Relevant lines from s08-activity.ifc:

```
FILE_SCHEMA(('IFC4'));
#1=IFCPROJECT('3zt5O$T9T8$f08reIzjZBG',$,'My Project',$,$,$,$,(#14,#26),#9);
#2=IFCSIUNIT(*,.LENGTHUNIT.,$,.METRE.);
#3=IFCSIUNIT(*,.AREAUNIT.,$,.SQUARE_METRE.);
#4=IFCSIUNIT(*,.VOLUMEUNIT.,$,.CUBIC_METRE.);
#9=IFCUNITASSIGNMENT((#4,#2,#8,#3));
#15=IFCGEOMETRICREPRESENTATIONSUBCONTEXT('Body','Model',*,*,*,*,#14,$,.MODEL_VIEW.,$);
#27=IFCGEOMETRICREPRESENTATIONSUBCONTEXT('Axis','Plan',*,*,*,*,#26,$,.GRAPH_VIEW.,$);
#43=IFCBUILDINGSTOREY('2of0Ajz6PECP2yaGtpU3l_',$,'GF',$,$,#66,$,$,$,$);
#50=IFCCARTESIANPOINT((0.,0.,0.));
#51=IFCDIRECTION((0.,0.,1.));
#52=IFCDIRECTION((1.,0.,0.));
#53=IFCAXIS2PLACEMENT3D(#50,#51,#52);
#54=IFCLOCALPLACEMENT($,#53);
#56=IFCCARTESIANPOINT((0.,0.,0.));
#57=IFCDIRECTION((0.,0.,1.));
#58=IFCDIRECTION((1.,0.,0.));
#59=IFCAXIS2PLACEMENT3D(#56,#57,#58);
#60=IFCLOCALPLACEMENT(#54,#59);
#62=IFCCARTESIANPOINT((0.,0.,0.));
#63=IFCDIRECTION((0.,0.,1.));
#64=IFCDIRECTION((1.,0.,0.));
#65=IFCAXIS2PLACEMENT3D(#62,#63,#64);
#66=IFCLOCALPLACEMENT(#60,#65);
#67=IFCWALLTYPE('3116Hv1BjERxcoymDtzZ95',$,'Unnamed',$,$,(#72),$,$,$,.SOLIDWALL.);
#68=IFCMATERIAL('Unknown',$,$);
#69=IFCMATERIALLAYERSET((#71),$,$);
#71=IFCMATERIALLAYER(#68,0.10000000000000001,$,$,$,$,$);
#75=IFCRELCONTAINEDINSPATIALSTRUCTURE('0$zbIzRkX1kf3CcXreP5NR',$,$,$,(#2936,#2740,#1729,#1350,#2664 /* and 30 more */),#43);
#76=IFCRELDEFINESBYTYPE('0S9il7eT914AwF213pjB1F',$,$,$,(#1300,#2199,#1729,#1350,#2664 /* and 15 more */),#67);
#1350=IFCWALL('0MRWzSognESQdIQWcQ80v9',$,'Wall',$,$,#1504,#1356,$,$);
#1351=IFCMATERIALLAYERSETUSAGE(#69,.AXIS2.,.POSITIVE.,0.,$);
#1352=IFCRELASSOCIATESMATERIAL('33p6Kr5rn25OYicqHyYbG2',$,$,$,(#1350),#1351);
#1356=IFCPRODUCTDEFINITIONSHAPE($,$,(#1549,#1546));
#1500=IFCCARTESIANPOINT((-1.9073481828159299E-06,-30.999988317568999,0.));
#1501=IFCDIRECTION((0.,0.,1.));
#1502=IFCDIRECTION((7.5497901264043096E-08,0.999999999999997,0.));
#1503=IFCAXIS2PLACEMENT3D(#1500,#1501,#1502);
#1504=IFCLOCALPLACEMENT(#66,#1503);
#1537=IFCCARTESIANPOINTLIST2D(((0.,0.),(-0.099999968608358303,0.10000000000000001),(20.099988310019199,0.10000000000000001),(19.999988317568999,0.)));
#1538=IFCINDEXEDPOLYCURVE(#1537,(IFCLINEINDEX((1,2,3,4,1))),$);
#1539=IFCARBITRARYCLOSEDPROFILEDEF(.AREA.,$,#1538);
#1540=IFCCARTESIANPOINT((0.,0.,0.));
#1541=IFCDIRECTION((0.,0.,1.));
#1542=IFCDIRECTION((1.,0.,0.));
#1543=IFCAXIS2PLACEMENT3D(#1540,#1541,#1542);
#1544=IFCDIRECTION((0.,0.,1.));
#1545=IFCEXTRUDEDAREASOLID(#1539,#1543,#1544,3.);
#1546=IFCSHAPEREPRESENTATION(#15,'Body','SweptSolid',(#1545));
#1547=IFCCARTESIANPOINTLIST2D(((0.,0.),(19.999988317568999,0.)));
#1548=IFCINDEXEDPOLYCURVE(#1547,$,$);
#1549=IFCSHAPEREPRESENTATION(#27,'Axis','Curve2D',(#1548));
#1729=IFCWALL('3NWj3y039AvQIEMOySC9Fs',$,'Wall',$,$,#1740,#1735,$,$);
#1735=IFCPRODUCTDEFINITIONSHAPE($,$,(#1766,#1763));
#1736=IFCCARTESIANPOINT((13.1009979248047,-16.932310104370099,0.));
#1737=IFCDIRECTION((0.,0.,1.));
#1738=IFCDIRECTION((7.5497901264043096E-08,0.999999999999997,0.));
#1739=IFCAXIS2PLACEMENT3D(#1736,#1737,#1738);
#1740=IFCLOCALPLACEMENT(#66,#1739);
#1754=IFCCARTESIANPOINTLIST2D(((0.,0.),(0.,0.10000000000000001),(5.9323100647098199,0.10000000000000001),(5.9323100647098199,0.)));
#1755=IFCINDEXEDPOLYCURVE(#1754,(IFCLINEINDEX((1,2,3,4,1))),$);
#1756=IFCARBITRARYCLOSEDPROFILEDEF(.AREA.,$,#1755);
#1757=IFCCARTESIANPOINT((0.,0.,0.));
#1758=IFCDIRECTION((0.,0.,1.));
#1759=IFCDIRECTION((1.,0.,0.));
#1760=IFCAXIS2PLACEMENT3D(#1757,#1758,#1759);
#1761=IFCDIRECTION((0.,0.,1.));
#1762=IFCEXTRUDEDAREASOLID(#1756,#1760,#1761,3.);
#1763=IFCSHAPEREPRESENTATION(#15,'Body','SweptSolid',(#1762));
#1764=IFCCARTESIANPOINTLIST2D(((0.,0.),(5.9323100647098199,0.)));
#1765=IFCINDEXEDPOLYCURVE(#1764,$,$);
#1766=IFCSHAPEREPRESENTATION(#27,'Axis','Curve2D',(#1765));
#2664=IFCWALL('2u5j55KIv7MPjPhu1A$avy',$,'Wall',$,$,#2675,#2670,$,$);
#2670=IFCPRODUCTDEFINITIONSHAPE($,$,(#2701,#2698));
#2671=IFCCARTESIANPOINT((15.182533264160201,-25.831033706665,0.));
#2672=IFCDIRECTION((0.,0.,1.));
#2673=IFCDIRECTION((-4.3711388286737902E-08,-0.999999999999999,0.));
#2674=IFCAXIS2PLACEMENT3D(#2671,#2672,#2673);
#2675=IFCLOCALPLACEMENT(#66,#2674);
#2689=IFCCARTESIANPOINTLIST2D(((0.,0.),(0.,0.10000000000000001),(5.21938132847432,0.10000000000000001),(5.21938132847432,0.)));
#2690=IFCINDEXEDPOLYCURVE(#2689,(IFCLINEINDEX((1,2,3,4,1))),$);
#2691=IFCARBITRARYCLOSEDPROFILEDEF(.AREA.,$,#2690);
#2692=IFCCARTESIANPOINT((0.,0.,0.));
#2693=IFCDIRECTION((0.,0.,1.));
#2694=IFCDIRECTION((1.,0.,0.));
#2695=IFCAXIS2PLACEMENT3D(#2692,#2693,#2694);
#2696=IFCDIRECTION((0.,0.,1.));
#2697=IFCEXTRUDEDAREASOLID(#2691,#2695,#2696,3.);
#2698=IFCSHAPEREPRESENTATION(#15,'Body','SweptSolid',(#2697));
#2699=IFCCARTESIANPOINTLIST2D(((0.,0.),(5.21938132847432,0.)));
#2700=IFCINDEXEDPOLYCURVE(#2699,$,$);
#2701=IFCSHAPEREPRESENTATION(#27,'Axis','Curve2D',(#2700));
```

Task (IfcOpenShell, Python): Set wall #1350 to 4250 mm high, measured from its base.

```python
import ifcopenshell
import ifcopenshell.geom
import ifcopenshell.util.representation
import ifcopenshell.util.shape
import ifcopenshell.util.unit

model = ifcopenshell.open("s08-activity.ifc")
unit_scale = ifcopenshell.util.unit.calculate_unit_scale(model)
settings = ifcopenshell.geom.settings()


def volume(element):
    """Net volume in cubic metres, openings subtracted."""
    shape = ifcopenshell.geom.create_shape(settings, element)
    return ifcopenshell.util.shape.get_volume(shape.geometry)


wall = model.by_id(1350)
before = volume(wall)

body = ifcopenshell.util.representation.get_representation(wall, "Model", "Body")
solid = body.Items[0]
old_height = solid.Depth
solid.Depth = 4.25 / unit_scale
after = volume(wall)

print(f"height {old_height:g} -> {solid.Depth:g}, volume {before:.3f} -> {after:.3f} m3")

model.write("s08-activity_v2.ifc")
```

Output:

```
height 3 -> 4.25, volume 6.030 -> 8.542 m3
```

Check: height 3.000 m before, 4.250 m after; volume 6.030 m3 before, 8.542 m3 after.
